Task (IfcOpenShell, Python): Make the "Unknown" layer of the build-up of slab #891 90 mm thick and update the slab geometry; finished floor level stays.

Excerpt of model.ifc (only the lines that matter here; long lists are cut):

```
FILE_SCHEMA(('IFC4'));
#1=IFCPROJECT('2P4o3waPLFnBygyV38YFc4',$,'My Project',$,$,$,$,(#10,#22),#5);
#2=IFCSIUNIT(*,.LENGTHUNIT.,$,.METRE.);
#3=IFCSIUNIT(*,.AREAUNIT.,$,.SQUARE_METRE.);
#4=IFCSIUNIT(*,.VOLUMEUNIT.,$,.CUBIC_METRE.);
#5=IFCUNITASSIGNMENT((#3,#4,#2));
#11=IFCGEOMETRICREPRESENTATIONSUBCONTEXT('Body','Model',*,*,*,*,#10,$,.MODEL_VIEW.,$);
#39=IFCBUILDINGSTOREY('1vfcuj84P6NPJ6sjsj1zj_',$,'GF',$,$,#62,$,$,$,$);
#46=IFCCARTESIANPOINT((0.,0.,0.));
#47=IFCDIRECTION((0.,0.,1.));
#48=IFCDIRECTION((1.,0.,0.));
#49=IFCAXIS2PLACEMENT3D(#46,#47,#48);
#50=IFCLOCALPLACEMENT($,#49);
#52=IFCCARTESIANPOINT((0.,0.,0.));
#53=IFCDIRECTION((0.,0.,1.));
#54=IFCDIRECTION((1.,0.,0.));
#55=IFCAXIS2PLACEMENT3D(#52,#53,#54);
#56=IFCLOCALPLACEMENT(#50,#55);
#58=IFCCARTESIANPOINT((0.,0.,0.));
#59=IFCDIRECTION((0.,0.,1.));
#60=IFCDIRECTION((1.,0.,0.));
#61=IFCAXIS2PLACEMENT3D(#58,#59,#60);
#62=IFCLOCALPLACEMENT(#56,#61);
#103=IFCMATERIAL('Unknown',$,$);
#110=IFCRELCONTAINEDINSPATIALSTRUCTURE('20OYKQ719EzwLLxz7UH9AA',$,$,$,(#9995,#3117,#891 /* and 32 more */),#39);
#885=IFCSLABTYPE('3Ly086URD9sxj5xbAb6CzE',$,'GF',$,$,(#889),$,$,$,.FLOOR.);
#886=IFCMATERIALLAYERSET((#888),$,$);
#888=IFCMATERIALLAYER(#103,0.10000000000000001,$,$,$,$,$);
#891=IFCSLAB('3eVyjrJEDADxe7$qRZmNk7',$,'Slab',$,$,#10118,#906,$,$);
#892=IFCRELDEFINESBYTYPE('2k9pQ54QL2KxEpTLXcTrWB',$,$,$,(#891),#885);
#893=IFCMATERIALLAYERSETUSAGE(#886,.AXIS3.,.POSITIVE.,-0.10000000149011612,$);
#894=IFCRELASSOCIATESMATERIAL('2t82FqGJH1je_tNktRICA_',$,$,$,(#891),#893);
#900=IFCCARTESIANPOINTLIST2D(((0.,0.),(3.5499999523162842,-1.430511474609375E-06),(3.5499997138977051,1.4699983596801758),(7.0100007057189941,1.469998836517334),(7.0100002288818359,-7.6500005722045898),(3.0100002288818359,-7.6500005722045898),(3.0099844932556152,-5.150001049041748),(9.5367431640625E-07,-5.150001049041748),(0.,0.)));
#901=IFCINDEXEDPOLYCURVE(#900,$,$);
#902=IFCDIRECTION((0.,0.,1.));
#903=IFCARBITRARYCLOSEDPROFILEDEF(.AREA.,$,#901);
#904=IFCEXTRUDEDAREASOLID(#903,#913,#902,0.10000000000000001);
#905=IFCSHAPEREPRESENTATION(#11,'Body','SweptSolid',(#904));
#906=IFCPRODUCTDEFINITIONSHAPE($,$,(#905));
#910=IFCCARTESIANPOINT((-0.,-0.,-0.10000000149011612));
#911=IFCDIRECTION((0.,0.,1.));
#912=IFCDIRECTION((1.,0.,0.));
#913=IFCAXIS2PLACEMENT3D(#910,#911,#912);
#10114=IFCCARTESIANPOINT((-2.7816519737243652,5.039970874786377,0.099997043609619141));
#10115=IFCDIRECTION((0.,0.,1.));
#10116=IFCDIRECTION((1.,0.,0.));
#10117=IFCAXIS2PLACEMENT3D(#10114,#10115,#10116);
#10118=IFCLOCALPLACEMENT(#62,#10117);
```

```python
import ifcopenshell
import ifcopenshell.util.element
import ifcopenshell.util.representation
import ifcopenshell.util.unit

model = ifcopenshell.open("model.ifc")
unit_scale = ifcopenshell.util.unit.calculate_unit_scale(model)

layer_set = model.by_id(886)
layer = next(l for l in layer_set.MaterialLayers if l.Material and l.Material.Name == "Unknown")
change = 0.09 / unit_scale - layer.LayerThickness
layer.LayerThickness += change

# Geometry does not follow the layer set by itself.
slabs = [e for e in ifcopenshell.util.element.get_elements_by_material(model, layer_set) if e.is_a("IfcSlab")]
for slab in sorted(slabs, key=lambda e: e.id()):
    body = ifcopenshell.util.representation.get_representation(slab, "Model", "Body")
    solid = body.Items[0]
    old_depth = solid.Depth
    solid.Depth += change
    # Extruded upwards: lower the start of the extrusion so the top stays.
    x, y, z = solid.Position.Location.Coordinates
    solid.Position.Location = model.createIfcCartesianPoint((x, y, z - change))
    print(slab.id(), f"{old_depth:g} -> {solid.Depth:g}")

# The layers are counted up from the underside, which has moved.
for usage in {ifcopenshell.util.element.get_material(slab) for slab in slabs}:
    usage.OffsetFromReferenceLine -= change

model.write("model-out.ifc")
```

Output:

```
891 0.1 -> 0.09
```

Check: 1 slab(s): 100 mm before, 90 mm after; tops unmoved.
